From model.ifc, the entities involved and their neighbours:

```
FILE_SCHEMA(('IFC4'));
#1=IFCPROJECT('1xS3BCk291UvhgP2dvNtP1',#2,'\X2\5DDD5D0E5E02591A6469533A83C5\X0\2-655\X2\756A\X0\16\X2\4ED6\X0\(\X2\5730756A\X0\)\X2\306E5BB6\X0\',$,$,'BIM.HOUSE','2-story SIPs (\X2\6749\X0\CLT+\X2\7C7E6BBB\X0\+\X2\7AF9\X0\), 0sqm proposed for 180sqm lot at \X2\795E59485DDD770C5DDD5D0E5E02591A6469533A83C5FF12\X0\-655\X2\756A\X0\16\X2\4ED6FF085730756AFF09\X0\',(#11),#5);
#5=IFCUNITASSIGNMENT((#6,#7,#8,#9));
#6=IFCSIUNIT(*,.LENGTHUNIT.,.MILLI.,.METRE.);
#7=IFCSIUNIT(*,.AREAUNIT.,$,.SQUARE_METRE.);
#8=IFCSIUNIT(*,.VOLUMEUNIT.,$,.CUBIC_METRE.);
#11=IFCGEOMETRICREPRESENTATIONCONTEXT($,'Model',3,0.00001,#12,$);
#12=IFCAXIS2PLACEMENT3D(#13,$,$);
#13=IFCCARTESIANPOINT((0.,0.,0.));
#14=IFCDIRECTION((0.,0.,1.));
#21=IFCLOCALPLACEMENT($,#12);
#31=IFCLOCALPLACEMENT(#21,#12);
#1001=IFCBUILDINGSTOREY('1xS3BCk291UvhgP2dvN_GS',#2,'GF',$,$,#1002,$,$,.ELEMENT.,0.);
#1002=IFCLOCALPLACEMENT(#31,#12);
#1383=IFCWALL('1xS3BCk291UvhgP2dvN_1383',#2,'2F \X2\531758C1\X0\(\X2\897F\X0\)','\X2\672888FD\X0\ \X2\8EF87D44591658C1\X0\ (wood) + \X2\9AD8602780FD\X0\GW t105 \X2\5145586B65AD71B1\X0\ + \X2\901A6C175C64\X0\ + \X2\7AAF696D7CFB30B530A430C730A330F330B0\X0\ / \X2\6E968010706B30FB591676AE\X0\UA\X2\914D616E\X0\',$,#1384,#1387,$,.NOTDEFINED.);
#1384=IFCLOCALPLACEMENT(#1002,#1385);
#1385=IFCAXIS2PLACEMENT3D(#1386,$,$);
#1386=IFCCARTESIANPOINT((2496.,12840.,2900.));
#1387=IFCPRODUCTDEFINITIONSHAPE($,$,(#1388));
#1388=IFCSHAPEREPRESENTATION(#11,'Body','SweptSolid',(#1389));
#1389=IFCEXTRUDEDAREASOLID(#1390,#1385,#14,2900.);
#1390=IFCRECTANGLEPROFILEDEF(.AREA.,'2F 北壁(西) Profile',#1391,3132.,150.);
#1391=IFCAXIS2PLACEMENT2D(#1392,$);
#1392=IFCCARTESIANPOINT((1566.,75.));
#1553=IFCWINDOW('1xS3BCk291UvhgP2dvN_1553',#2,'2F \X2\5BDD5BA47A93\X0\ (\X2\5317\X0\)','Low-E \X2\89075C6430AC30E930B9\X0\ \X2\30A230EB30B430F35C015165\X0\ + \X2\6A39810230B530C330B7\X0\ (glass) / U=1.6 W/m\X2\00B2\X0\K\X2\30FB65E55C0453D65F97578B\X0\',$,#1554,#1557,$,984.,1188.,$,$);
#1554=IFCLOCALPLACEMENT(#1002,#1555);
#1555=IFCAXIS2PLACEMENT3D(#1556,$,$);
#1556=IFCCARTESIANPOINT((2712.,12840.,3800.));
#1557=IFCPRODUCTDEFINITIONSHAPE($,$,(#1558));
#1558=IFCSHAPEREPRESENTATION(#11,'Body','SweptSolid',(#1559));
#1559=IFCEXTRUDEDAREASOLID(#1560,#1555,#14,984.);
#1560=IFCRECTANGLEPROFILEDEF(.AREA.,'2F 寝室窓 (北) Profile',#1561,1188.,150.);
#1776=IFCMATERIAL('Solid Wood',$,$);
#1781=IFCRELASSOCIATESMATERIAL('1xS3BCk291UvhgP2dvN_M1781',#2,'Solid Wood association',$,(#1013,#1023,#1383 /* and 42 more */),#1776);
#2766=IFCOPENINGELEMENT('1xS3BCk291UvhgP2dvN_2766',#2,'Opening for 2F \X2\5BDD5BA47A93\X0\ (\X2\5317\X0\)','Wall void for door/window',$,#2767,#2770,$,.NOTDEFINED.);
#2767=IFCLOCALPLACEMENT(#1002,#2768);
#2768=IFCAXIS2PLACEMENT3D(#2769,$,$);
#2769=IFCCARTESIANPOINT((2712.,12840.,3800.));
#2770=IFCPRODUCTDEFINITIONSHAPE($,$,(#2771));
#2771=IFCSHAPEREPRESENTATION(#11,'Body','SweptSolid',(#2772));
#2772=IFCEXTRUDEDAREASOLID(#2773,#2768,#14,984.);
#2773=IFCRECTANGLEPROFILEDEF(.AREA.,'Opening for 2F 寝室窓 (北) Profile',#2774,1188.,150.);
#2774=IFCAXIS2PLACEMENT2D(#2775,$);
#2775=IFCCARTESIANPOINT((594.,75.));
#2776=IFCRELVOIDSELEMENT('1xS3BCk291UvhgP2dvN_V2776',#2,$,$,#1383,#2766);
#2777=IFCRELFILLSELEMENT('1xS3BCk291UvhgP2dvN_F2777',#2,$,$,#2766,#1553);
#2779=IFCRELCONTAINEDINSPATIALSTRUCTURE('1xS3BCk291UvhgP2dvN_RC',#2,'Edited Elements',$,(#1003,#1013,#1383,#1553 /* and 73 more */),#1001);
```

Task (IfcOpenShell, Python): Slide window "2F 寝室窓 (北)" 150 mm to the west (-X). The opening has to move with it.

```python
import ifcopenshell
import ifcopenshell.api.geometry
import ifcopenshell.util.placement

model = ifcopenshell.open("model.ifc")

window = model.by_guid("1xS3BCk291UvhgP2dvN_1553")
opening = window.FillsVoids[0].RelatingOpeningElement
wall = opening.VoidsElements[0].RelatingBuildingElement

wall_matrix = ifcopenshell.util.placement.get_local_placement(wall.ObjectPlacement)
shift = wall_matrix[:3, 0] * -150.0
before = ifcopenshell.util.placement.get_local_placement(window.ObjectPlacement)[:3, 3].copy()

# The window is not placed relative to its opening, so move both.
for product in (opening, window):
    matrix = ifcopenshell.util.placement.get_local_placement(product.ObjectPlacement)
    matrix[:3, 3] += shift
    ifcopenshell.api.geometry.edit_object_placement(model, product=product, matrix=matrix, is_si=False)

after = ifcopenshell.util.placement.get_local_placement(window.ObjectPlacement)[:3, 3]
print("window moved by", (after - before).round(3) + 0.0)

model.write("model-out.ifc")
```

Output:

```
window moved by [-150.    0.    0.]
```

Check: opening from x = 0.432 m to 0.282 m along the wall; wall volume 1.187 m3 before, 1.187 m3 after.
